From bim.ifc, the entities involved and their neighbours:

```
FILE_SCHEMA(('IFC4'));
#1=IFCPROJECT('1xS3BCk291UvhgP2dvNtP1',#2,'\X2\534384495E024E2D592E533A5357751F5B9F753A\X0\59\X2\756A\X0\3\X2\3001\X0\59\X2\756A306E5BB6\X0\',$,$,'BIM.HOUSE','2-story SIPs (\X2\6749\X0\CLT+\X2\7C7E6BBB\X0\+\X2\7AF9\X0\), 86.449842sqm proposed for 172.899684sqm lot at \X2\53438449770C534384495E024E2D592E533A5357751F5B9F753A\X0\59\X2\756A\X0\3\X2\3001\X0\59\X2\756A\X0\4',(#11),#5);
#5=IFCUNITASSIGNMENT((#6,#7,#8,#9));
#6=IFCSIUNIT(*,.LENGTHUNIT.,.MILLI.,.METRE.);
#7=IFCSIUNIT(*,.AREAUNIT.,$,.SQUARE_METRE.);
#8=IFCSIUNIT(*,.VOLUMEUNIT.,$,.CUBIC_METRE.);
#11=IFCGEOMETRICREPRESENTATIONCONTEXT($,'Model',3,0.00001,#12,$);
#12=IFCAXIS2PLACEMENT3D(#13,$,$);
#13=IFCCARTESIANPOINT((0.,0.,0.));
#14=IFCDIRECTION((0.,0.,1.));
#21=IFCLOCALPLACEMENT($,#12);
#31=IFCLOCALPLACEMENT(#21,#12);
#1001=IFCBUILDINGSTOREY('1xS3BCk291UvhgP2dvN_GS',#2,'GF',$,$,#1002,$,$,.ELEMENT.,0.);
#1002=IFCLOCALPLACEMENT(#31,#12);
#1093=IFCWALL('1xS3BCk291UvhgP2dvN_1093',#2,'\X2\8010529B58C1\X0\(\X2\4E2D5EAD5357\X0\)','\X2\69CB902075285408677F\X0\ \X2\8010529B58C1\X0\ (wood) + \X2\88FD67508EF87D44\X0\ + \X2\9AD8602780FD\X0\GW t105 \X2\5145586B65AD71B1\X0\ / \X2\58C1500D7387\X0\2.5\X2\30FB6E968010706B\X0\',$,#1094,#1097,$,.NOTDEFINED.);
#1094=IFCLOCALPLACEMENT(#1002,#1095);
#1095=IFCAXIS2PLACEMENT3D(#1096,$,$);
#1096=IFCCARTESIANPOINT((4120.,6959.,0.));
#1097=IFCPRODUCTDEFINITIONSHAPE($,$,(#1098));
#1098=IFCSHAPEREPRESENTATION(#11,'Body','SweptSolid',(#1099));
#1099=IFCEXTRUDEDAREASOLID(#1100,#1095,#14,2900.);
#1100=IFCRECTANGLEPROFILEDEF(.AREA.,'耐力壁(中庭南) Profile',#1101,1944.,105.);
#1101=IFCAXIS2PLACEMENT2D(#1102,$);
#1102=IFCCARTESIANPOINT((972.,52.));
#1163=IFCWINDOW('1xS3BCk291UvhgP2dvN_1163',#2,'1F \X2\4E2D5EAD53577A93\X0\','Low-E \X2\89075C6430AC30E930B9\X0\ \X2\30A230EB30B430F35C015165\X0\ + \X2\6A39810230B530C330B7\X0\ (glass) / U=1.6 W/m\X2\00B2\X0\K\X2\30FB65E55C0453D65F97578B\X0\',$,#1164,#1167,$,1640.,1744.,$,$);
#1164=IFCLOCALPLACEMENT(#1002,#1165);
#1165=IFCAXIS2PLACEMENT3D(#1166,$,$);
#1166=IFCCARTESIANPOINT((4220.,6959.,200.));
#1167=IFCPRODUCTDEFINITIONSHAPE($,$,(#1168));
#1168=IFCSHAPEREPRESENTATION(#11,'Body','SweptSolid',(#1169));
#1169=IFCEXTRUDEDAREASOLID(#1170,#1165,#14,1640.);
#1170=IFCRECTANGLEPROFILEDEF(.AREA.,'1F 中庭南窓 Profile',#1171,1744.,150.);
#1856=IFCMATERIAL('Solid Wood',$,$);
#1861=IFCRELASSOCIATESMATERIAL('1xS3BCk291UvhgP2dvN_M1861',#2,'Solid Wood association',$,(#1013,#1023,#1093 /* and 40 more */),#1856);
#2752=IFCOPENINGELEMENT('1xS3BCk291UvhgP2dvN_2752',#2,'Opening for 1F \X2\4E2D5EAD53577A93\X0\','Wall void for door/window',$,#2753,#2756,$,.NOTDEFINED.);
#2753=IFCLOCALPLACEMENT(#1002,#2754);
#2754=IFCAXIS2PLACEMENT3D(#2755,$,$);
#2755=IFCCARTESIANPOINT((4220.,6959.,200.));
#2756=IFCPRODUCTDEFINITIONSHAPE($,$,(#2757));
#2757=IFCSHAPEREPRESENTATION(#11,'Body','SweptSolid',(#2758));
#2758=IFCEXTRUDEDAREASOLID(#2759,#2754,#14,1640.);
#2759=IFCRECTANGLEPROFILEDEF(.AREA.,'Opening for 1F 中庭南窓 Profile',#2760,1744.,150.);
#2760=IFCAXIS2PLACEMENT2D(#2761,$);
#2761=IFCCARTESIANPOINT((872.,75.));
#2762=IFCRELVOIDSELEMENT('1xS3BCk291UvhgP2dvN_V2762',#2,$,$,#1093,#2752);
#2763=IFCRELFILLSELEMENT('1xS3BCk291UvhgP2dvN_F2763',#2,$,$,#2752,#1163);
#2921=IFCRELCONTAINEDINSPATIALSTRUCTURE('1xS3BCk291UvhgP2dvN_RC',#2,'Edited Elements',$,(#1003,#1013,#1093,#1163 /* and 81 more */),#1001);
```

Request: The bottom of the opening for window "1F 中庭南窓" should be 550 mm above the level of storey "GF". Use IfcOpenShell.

```python
import numpy as np
import ifcopenshell
import ifcopenshell.api.geometry
import ifcopenshell.geom
import ifcopenshell.util.element
import ifcopenshell.util.placement
import ifcopenshell.util.shape
import ifcopenshell.util.unit

model = ifcopenshell.open("bim.ifc")
unit_scale = ifcopenshell.util.unit.calculate_unit_scale(model)

window = model.by_guid("1xS3BCk291UvhgP2dvN_1163")
opening = window.FillsVoids[0].RelatingOpeningElement
storey = ifcopenshell.util.element.get_container(window, ifc_class="IfcBuildingStorey")
level = ifcopenshell.util.placement.get_local_placement(storey.ObjectPlacement)[2, 3]

# The opening's origin need not be at the sill, so measure its lowest point.
shape = ifcopenshell.geom.create_shape(ifcopenshell.geom.settings(), opening)
bottom = ifcopenshell.util.shape.get_shape_bottom_elevation(shape, shape.geometry) / unit_scale
dz = level + 550.0 - bottom

shift = np.array([0.0, 0.0, dz])
# The window is not placed relative to its opening, so move both.
for product in (opening, window):
    matrix = ifcopenshell.util.placement.get_local_placement(product.ObjectPlacement)
    matrix[:3, 3] += shift
    ifcopenshell.api.geometry.edit_object_placement(model, product=product, matrix=matrix, is_si=False)

print(f"moved by {dz * unit_scale:+.3f} m")

model.write("bim_edited.ifc")
```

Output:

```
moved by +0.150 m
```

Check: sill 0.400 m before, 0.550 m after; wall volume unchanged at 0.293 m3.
